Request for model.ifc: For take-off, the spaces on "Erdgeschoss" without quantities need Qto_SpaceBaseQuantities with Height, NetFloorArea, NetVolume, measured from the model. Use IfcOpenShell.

First a look at what the model holds.

```python
import ifcopenshell
import ifcopenshell.util.element
import ifcopenshell.util.unit

model = ifcopenshell.open("model.ifc")
print(model.schema)
for unit_type in ("LENGTHUNIT", "AREAUNIT", "VOLUMEUNIT"):
    print(unit_type, ifcopenshell.util.unit.calculate_unit_scale(model, unit_type))
storey = next(s for s in model.by_type("IfcBuildingStorey") if s.Name == "Erdgeschoss")
spaces = [e for e in ifcopenshell.util.element.get_decomposition(storey) if e.is_a("IfcSpace")]
for e in sorted(spaces, key=lambda e: e.id()):
    print(e.id(), e.is_a(), e.Name, list(ifcopenshell.util.element.get_psets(e, qtos_only=True)), sep=" | ")
```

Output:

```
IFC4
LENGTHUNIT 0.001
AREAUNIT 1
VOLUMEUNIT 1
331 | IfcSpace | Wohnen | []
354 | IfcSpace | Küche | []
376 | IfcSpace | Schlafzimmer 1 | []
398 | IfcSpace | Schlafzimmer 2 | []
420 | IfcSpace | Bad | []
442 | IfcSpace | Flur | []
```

```python
import ifcopenshell
import ifcopenshell.api.pset
import ifcopenshell.geom
import ifcopenshell.util.element
import ifcopenshell.util.shape
import ifcopenshell.util.unit

model = ifcopenshell.open("model.ifc")
unit_scale = ifcopenshell.util.unit.calculate_unit_scale(model)
area_scale = ifcopenshell.util.unit.calculate_unit_scale(model, "AREAUNIT")
volume_scale = ifcopenshell.util.unit.calculate_unit_scale(model, "VOLUMEUNIT")
settings = ifcopenshell.geom.settings()

storey = next(s for s in model.by_type("IfcBuildingStorey") if s.Name == "Erdgeschoss")
spaces = [e for e in ifcopenshell.util.element.get_decomposition(storey) if e.is_a("IfcSpace")]

for e in sorted(spaces, key=lambda e: e.id()):
    if ifcopenshell.util.element.get_psets(e, qtos_only=True, should_inherit=False):
        continue
    # Geometry comes back in metres, in the element's own axes.
    shape = ifcopenshell.geom.create_shape(settings, e)
    values = {
        "Height": ifcopenshell.util.shape.get_z(shape.geometry) / unit_scale,
        "NetFloorArea": ifcopenshell.util.shape.get_footprint_area(shape.geometry) / area_scale,
        "NetVolume": ifcopenshell.util.shape.get_volume(shape.geometry) / volume_scale,
    }
    qto = ifcopenshell.api.pset.add_qto(model, product=e, name="Qto_SpaceBaseQuantities")
    ifcopenshell.api.pset.edit_qto(model, qto=qto, properties=values)
    print(e.id(), {k: round(v, 3) for k, v in values.items()})

model.write("model_updated.ifc")
```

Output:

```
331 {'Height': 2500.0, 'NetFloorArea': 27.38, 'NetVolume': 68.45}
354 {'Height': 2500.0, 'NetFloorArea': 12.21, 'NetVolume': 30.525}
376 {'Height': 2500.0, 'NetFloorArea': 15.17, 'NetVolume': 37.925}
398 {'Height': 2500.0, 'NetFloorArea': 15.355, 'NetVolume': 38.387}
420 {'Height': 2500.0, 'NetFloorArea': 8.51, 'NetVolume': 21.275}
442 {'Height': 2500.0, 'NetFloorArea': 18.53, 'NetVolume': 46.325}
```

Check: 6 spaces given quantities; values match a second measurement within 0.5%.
